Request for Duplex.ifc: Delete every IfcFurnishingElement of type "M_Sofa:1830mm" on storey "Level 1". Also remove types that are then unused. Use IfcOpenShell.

First a look at what the model holds.

```python
import ifcopenshell
import ifcopenshell.util.element

model = ifcopenshell.open("Duplex.ifc")
print(model.schema)
storey = next(s for s in model.by_type("IfcBuildingStorey") if s.Name == "Level 1")
furniture = [e for e in ifcopenshell.util.element.get_decomposition(storey) if e.is_a("IfcFurnishingElement")]
seen = {}
for e in furniture:
    element_type = ifcopenshell.util.element.get_type(e)
    name = element_type.Name if element_type not in (None, e) else None
    seen[name] = seen.get(name, 0) + 1
for name, count in sorted(seen.items(), key=str):
    print(count, "x", name)
```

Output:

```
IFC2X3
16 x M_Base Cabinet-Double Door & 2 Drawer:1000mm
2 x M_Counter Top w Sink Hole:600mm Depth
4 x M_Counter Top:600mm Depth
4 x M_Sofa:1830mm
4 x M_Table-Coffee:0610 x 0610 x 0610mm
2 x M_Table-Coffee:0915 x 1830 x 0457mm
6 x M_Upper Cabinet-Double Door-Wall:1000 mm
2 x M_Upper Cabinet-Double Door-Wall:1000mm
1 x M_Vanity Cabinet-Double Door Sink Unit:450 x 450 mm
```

```python
import ifcopenshell
import ifcopenshell.api.root
import ifcopenshell.util.element

model = ifcopenshell.open("Duplex.ifc")

storey = next(s for s in model.by_type("IfcBuildingStorey") if s.Name == "Level 1")
furniture = [e for e in ifcopenshell.util.element.get_decomposition(storey) if e.is_a("IfcFurnishingElement")]
targets = [e for e in furniture if (t := ifcopenshell.util.element.get_type(e)) not in (None, e) and t.Name == "M_Sofa:1830mm"]
types = {ifcopenshell.util.element.get_type(e) for e in targets} - {None, *targets}

for e in targets:
    ifcopenshell.api.root.remove_product(model, product=e)
print(len(targets), "removed")

unused = [t for t in types if not ifcopenshell.util.element.get_types(t)]
for t in unused:
    ifcopenshell.api.root.remove_product(model, product=t)
print(len(unused), "unused types removed")

model.write("Duplex_rev.ifc")
```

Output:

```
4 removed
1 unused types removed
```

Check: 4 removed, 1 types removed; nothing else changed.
